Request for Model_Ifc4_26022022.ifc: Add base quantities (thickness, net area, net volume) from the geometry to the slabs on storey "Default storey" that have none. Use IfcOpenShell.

First a look at what the model holds.

```python
import ifcopenshell
import ifcopenshell.util.element
import ifcopenshell.util.unit

model = ifcopenshell.open("Model_Ifc4_26022022.ifc")
print(model.schema)
for unit_type in ("LENGTHUNIT", "AREAUNIT", "VOLUMEUNIT"):
    print(unit_type, ifcopenshell.util.unit.calculate_unit_scale(model, unit_type))
storey = next(s for s in model.by_type("IfcBuildingStorey") if s.Name == "Default storey")
slabs = [e for e in ifcopenshell.util.element.get_decomposition(storey) if e.is_a("IfcSlab")]
for e in sorted(slabs, key=lambda e: e.id()):
    print(e.id(), e.is_a(), e.Name, list(ifcopenshell.util.element.get_psets(e, qtos_only=True)), sep=" | ")
```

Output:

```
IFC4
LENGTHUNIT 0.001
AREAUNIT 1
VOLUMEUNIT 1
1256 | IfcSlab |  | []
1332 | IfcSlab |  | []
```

```python
import ifcopenshell
import ifcopenshell.api.pset
import ifcopenshell.geom
import ifcopenshell.util.element
import ifcopenshell.util.shape
import ifcopenshell.util.unit

model = ifcopenshell.open("Model_Ifc4_26022022.ifc")
unit_scale = ifcopenshell.util.unit.calculate_unit_scale(model)
area_scale = ifcopenshell.util.unit.calculate_unit_scale(model, "AREAUNIT")
volume_scale = ifcopenshell.util.unit.calculate_unit_scale(model, "VOLUMEUNIT")
settings = ifcopenshell.geom.settings()

storey = next(s for s in model.by_type("IfcBuildingStorey") if s.Name == "Default storey")
slabs = [e for e in ifcopenshell.util.element.get_decomposition(storey) if e.is_a("IfcSlab")]

for e in sorted(slabs, key=lambda e: e.id()):
    if ifcopenshell.util.element.get_psets(e, qtos_only=True, should_inherit=False):
        continue
    # Geometry comes back in metres, in the element's own axes.
    shape = ifcopenshell.geom.create_shape(settings, e)
    values = {
        "Width": ifcopenshell.util.shape.get_z(shape.geometry) / unit_scale,
        "NetArea": ifcopenshell.util.shape.get_footprint_area(shape.geometry) / area_scale,
        "NetVolume": ifcopenshell.util.shape.get_volume(shape.geometry) / volume_scale,
    }
    qto = ifcopenshell.api.pset.add_qto(model, product=e, name="Qto_SlabBaseQuantities")
    ifcopenshell.api.pset.edit_qto(model, qto=qto, properties=values)
    print(e.id(), {k: round(v, 3) for k, v in values.items()})

model.write("Model_Ifc4_26022022_rev.ifc")
```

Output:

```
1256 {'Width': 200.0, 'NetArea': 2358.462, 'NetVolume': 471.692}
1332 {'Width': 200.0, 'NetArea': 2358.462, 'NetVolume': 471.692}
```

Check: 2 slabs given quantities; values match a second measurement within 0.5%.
